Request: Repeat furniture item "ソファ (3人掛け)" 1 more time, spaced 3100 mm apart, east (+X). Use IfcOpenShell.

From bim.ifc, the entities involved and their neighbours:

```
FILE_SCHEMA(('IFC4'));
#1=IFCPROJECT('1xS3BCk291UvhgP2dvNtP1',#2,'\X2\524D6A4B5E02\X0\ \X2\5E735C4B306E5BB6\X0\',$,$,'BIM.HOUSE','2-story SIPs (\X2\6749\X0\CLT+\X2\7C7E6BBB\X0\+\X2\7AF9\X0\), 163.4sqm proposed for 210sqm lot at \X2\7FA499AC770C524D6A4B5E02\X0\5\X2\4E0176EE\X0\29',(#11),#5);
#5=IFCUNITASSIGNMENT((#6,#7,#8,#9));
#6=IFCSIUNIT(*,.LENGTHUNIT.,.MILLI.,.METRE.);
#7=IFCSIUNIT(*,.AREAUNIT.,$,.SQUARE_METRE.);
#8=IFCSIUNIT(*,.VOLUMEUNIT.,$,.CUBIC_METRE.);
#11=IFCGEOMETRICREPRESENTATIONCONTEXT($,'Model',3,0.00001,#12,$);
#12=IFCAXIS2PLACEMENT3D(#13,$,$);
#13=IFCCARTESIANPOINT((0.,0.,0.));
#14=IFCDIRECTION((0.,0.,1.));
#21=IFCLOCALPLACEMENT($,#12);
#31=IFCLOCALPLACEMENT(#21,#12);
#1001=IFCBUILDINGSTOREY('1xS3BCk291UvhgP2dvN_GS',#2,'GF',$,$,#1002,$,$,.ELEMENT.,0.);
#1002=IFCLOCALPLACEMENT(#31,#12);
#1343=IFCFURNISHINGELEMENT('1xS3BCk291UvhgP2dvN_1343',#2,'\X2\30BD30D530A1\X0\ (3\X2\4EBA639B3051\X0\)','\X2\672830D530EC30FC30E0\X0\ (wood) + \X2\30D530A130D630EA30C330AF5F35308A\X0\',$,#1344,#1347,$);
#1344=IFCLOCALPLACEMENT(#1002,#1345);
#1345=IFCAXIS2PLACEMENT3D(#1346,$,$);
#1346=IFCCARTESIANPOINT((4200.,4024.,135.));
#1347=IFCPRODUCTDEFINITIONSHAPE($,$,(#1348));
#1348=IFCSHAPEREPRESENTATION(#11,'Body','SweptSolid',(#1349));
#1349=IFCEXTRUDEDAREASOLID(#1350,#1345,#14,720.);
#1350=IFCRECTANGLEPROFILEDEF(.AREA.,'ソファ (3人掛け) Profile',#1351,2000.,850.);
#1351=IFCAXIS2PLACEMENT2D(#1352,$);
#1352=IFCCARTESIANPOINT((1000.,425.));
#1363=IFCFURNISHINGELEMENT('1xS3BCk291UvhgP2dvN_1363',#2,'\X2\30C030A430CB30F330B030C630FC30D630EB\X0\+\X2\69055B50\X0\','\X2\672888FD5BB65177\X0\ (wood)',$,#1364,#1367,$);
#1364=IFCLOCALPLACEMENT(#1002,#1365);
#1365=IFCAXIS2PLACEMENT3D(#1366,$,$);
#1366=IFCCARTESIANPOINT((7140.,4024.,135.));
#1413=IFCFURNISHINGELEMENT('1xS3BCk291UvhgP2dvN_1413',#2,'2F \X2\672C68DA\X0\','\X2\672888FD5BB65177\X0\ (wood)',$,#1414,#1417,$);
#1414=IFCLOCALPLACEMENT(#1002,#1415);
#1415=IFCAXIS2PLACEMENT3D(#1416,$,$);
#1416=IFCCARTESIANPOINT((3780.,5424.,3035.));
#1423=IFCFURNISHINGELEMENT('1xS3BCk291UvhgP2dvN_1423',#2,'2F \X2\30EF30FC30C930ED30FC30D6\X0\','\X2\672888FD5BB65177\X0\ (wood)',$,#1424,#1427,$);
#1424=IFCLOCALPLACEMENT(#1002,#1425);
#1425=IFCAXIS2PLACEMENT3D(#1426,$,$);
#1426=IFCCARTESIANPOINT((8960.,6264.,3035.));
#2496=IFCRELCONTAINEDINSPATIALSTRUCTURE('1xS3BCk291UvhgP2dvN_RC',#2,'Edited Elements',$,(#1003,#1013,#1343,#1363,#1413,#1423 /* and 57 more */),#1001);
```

```python
import numpy as np
import ifcopenshell
import ifcopenshell.api.geometry
import ifcopenshell.api.root
import ifcopenshell.util.element
import ifcopenshell.util.placement
import ifcopenshell.util.unit

model = ifcopenshell.open("bim.ifc")
unit_scale = ifcopenshell.util.unit.calculate_unit_scale(model)


def reuse_history(source, copy):
    """copy_class also copies each property set's owner history, people and application; keep the originals."""
    for rel in copy.IsDefinedBy:
        if rel.is_a("IfcRelDefinesByProperties") and (history := rel.RelatingPropertyDefinition.OwnerHistory):
            rel.RelatingPropertyDefinition.OwnerHistory = source.OwnerHistory
            ifcopenshell.util.element.remove_deep2(model, history)


source = model.by_id(1343)
base = ifcopenshell.util.placement.get_local_placement(source.ObjectPlacement)
step = np.array([1.0, 0.0, 0.0]) * 3.1 / unit_scale

for i in range(1, 2):
    copy = ifcopenshell.api.root.copy_class(model, product=source)
    copy.Representation = ifcopenshell.util.element.copy_deep(
        model, source.Representation, exclude=["IfcGeometricRepresentationContext", "IfcRepresentationMap"]
    )
    reuse_history(source, copy)
    matrix = base.copy()
    matrix[:3, 3] += i * step
    print("added at", matrix[:3, 3].round(3) + 0.0)
    ifcopenshell.api.geometry.edit_object_placement(model, product=copy, matrix=matrix, is_si=False)

model.write("bim_edited.ifc")
```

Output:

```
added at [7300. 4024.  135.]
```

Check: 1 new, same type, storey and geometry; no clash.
